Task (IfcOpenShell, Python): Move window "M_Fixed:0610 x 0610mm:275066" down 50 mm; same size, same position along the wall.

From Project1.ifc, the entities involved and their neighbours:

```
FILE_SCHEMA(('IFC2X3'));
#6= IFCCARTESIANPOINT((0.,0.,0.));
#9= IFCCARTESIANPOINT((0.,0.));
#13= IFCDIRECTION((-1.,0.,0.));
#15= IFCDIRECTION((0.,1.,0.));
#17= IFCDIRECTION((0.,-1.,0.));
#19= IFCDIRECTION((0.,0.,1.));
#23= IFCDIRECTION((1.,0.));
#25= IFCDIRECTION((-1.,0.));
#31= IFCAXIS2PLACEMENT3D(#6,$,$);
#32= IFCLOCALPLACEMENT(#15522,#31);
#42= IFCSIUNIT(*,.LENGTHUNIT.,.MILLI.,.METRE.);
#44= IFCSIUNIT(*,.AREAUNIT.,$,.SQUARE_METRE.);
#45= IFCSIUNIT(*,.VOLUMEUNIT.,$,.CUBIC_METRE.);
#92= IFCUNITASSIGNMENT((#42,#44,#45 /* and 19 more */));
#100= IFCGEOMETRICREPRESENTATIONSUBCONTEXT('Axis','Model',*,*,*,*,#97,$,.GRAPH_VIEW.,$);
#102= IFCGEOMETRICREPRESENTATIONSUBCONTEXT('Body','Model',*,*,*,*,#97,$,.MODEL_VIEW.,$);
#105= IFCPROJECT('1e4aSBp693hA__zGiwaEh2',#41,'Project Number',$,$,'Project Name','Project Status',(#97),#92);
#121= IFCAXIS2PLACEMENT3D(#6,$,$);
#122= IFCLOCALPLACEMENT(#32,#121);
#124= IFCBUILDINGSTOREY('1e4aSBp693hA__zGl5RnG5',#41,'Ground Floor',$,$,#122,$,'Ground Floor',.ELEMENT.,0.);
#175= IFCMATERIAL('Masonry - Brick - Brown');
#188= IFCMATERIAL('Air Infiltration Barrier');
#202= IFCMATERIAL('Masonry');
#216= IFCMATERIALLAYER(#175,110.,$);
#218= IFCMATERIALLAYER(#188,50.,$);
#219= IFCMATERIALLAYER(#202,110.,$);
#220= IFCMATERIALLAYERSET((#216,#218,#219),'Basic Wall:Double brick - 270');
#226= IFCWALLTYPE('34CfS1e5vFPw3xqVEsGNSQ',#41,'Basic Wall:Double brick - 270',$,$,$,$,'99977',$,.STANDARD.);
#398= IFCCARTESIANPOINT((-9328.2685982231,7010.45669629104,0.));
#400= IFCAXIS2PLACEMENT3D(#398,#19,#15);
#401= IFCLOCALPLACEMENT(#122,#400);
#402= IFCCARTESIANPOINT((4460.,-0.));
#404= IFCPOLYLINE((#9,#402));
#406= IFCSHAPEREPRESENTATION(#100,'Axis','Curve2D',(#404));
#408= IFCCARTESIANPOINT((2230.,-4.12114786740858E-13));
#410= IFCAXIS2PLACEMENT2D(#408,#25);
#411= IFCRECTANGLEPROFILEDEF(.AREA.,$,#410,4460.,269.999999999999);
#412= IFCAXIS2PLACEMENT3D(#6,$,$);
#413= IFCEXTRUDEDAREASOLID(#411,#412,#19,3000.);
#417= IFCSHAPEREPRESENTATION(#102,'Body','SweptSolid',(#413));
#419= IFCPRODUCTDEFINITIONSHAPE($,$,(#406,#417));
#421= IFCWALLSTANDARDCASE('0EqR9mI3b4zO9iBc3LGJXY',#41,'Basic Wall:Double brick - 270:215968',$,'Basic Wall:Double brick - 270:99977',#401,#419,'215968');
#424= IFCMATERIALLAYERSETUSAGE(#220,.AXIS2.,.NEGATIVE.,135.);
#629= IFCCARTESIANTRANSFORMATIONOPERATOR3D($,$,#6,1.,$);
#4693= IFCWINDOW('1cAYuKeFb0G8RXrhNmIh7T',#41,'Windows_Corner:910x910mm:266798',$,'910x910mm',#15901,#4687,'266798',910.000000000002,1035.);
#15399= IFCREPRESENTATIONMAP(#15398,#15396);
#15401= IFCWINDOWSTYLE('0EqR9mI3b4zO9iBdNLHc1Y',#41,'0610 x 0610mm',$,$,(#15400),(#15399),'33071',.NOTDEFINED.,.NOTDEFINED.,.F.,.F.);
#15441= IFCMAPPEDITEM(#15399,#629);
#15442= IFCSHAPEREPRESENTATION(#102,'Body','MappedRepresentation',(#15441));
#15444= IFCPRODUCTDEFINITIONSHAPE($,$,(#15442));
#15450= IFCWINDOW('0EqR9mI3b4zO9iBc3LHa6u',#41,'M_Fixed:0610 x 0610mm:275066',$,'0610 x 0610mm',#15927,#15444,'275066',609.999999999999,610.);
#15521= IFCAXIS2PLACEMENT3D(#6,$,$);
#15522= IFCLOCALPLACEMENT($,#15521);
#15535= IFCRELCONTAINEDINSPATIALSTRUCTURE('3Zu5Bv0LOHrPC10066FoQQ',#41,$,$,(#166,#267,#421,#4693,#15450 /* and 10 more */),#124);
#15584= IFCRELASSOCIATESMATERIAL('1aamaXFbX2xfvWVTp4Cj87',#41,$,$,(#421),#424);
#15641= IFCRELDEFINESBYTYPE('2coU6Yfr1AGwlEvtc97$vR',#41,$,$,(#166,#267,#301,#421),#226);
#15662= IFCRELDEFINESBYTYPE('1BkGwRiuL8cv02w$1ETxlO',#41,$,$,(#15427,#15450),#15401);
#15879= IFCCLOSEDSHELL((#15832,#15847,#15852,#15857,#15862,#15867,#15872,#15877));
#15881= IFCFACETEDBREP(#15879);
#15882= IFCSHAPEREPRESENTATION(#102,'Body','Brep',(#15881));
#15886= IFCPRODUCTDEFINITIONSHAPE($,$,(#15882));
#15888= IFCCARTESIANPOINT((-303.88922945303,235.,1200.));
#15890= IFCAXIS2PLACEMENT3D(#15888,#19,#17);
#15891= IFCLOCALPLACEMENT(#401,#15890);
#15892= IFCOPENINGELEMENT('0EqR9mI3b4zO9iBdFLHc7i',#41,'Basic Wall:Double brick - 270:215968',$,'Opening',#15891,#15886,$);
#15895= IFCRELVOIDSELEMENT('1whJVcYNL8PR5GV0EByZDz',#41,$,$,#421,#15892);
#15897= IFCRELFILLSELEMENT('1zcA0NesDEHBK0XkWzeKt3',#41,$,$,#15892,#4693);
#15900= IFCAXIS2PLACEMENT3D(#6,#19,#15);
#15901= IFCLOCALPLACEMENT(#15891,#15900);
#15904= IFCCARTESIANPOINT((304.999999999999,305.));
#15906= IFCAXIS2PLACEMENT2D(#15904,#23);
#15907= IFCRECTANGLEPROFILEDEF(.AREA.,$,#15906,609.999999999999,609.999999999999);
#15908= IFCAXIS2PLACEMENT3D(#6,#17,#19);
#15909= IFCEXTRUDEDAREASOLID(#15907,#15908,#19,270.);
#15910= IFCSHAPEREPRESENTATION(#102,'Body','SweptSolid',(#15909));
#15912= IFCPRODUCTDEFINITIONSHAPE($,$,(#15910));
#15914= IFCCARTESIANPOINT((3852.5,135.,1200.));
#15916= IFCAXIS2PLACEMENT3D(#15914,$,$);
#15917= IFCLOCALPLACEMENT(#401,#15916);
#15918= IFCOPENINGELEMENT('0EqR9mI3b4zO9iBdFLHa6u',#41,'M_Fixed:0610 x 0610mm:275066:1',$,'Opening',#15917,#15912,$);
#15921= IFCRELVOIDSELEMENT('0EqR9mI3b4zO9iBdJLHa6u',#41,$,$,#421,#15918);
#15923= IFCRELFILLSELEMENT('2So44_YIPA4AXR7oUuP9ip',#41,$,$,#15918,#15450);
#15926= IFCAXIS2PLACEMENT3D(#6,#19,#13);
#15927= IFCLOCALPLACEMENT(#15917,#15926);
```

```python
import numpy as np
import ifcopenshell
import ifcopenshell.api.geometry
import ifcopenshell.util.placement
import ifcopenshell.util.unit

model = ifcopenshell.open("Project1.ifc")
unit_scale = ifcopenshell.util.unit.calculate_unit_scale(model)

window = model.by_guid("0EqR9mI3b4zO9iBc3LHa6u")
opening = window.FillsVoids[0].RelatingOpeningElement
dz = -0.05 / unit_scale

shift = np.array([0.0, 0.0, dz])
# The window is placed relative to its opening, so it follows when the opening moves.
matrix = ifcopenshell.util.placement.get_local_placement(opening.ObjectPlacement)
matrix[:3, 3] += shift
ifcopenshell.api.geometry.edit_object_placement(
    model, product=opening, matrix=matrix, is_si=False, should_transform_children=True
)

print(f"moved by {dz * unit_scale:+.3f} m")

model.write("Project1_v2.ifc")
```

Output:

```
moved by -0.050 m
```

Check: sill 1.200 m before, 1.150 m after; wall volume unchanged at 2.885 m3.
